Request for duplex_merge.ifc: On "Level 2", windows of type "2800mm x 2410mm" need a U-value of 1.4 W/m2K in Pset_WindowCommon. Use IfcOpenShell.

First a look at what the model holds.

```python
import ifcopenshell
import ifcopenshell.util.element

model = ifcopenshell.open("duplex_merge.ifc")
print(model.schema)
storey = next(s for s in model.by_type("IfcBuildingStorey") if s.Name == "Level 2")
windows = [e for e in ifcopenshell.util.element.get_decomposition(storey) if e.is_a("IfcWindow")]
seen = {}
for e in windows:
    element_type = ifcopenshell.util.element.get_type(e)
    key = (element_type.Name if element_type != e and element_type else None, ifcopenshell.util.element.get_pset(e, "Pset_WindowCommon", "ThermalTransmittance"))
    seen[key] = seen.get(key, 0) + 1
for (name, value), count in sorted(seen.items(), key=str):
    print(count, "x", name, "|", value)
```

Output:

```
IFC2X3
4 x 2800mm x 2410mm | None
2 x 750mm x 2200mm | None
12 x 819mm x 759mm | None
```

```python
import ifcopenshell
import ifcopenshell.api.pset
import ifcopenshell.util.element

model = ifcopenshell.open("duplex_merge.ifc")

storey = next(s for s in model.by_type("IfcBuildingStorey") if s.Name == "Level 2")
windows = [e for e in ifcopenshell.util.element.get_decomposition(storey) if e.is_a("IfcWindow")]

count = 0
for e in windows:
    element_type = ifcopenshell.util.element.get_type(e)
    if element_type in (None, e) or element_type.Name != "2800mm x 2410mm":
        continue
    # add_pset returns the element's existing set when there is one.
    pset = ifcopenshell.api.pset.add_pset(model, product=e, name="Pset_WindowCommon")
    ifcopenshell.api.pset.edit_pset(model, pset=pset, properties={"ThermalTransmittance": 1.4})
    count += 1

print(count, "windows updated")

model.write("duplex_merge_v2.ifc")
```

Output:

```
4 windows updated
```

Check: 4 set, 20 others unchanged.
